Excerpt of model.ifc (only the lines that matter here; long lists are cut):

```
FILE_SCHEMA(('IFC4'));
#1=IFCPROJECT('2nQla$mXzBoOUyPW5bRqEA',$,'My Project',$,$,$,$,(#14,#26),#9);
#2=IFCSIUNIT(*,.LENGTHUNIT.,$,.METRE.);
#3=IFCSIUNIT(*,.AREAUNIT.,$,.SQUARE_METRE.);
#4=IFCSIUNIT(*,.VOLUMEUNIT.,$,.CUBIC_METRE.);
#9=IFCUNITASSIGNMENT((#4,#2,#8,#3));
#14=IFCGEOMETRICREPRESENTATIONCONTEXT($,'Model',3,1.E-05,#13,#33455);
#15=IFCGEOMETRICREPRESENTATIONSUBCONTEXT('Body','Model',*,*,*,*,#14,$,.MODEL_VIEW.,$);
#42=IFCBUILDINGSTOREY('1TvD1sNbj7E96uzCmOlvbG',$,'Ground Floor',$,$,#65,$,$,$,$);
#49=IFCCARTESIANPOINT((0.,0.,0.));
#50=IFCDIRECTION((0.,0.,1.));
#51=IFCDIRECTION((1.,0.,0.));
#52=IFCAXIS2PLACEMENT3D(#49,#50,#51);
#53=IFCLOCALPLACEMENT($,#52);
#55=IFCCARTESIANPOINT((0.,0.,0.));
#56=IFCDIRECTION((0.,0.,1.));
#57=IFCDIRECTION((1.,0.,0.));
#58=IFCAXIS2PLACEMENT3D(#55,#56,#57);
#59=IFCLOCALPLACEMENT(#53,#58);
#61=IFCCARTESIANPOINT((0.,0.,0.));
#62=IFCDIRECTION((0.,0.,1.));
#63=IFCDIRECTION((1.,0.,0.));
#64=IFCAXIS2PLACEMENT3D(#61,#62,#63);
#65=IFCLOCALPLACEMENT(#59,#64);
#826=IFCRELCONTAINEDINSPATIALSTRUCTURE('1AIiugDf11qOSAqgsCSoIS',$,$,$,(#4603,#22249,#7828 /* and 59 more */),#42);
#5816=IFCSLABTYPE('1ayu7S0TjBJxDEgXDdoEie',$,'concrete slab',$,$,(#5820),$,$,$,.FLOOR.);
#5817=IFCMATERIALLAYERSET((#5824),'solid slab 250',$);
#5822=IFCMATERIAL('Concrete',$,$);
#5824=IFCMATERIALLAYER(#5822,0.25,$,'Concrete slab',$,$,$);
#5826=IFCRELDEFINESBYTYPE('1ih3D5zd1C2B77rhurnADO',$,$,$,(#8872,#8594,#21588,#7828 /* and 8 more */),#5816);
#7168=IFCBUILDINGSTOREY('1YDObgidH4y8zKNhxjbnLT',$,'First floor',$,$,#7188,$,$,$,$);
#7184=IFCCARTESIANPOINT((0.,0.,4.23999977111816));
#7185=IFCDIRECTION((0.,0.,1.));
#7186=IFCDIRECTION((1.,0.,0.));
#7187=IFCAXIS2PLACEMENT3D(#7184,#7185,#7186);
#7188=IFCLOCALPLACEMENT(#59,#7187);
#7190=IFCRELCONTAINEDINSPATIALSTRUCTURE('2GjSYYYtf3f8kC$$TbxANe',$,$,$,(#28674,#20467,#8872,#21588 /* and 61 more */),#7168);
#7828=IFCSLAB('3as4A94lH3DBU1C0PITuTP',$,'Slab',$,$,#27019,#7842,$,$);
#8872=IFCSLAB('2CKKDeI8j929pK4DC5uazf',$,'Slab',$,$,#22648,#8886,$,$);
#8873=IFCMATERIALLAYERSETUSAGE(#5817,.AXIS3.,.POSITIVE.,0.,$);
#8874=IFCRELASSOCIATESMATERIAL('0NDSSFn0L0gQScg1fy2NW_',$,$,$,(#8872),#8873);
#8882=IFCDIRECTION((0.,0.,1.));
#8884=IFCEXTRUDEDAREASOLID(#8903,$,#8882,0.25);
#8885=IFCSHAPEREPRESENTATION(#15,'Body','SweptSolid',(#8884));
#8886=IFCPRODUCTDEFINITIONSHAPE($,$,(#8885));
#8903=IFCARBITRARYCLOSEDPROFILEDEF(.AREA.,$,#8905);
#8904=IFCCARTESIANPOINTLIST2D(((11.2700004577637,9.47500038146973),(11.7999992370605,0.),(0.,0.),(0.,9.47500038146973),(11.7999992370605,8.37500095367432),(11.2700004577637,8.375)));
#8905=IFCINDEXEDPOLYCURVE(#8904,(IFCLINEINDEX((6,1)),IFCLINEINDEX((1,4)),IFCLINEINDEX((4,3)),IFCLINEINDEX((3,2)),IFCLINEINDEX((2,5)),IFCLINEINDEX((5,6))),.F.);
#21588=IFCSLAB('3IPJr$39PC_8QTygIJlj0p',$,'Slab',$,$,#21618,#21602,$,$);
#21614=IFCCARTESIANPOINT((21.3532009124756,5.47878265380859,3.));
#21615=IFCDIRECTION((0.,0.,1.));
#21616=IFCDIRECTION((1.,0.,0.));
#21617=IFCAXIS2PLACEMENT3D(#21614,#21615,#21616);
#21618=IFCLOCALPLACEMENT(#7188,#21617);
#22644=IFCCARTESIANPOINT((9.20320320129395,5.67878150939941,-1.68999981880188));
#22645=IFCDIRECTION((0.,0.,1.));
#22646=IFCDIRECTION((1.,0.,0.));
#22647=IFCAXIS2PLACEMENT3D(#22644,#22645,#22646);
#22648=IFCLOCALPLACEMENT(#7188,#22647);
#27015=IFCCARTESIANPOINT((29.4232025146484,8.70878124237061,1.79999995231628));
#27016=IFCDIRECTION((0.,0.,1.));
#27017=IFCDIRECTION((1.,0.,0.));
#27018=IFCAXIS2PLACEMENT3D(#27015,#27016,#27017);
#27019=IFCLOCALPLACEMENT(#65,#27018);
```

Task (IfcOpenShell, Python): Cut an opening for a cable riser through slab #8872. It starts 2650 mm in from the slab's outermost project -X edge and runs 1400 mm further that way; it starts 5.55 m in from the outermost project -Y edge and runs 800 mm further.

```python
import numpy as np
import ifcopenshell
import ifcopenshell.api.feature
import ifcopenshell.api.geometry
import ifcopenshell.api.root
import ifcopenshell.geom
import ifcopenshell.util.placement
import ifcopenshell.util.representation
import ifcopenshell.util.shape
import ifcopenshell.util.unit

model = ifcopenshell.open("model.ifc")
unit_scale = ifcopenshell.util.unit.calculate_unit_scale(model)
settings = ifcopenshell.geom.settings()


def volume(element):
    """Net volume in cubic metres, openings subtracted."""
    shape = ifcopenshell.geom.create_shape(settings, element)
    return ifcopenshell.util.shape.get_volume(shape.geometry)


slab = model.by_guid("2CKKDeI8j929pK4DC5uazf")
before = volume(slab)

# Extent in the slab's own axes, in metres. The edges named are its -X and -Y sides.
slab_shape = ifcopenshell.geom.create_shape(settings, slab)
vertices = ifcopenshell.util.shape.get_vertices(slab_shape.geometry)
x_min, y_min, bottom = vertices.min(axis=0)
top = vertices[:, 2].max()

opening = ifcopenshell.api.root.create_entity(model, ifc_class="IfcOpeningElement", name="Cable riser opening", predefined_type="OPENING")
context = ifcopenshell.util.representation.get_context(model, "Model", "Body", "MODEL_VIEW")
width, depth = 1.4, 0.8
outline = [(0.0, 0.0), (width, 0.0), (width, depth), (0.0, depth), (0.0, 0.0)]
# Overshoot both faces by 50 mm so the cut is clean.
shape = ifcopenshell.api.geometry.add_slab_representation(
    model, context=context, depth=top - bottom + 0.1, polyline=outline
)
ifcopenshell.api.geometry.assign_representation(model, product=opening, representation=shape)

matrix = ifcopenshell.util.placement.get_local_placement(slab.ObjectPlacement)
matrix[:, 3] = matrix @ np.append(np.array([x_min + 2.65, y_min + 5.55, bottom - 0.05]) / unit_scale, 1.0)
ifcopenshell.api.geometry.edit_object_placement(model, product=opening, matrix=matrix, is_si=False)
ifcopenshell.api.feature.add_feature(model, feature=opening, element=slab)

after = volume(slab)

print(f"slab volume {before:.3f} -> {after:.3f} m3")

model.write("model_edited.ifc")
```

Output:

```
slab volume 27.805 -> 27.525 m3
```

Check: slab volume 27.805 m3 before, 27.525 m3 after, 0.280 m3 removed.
